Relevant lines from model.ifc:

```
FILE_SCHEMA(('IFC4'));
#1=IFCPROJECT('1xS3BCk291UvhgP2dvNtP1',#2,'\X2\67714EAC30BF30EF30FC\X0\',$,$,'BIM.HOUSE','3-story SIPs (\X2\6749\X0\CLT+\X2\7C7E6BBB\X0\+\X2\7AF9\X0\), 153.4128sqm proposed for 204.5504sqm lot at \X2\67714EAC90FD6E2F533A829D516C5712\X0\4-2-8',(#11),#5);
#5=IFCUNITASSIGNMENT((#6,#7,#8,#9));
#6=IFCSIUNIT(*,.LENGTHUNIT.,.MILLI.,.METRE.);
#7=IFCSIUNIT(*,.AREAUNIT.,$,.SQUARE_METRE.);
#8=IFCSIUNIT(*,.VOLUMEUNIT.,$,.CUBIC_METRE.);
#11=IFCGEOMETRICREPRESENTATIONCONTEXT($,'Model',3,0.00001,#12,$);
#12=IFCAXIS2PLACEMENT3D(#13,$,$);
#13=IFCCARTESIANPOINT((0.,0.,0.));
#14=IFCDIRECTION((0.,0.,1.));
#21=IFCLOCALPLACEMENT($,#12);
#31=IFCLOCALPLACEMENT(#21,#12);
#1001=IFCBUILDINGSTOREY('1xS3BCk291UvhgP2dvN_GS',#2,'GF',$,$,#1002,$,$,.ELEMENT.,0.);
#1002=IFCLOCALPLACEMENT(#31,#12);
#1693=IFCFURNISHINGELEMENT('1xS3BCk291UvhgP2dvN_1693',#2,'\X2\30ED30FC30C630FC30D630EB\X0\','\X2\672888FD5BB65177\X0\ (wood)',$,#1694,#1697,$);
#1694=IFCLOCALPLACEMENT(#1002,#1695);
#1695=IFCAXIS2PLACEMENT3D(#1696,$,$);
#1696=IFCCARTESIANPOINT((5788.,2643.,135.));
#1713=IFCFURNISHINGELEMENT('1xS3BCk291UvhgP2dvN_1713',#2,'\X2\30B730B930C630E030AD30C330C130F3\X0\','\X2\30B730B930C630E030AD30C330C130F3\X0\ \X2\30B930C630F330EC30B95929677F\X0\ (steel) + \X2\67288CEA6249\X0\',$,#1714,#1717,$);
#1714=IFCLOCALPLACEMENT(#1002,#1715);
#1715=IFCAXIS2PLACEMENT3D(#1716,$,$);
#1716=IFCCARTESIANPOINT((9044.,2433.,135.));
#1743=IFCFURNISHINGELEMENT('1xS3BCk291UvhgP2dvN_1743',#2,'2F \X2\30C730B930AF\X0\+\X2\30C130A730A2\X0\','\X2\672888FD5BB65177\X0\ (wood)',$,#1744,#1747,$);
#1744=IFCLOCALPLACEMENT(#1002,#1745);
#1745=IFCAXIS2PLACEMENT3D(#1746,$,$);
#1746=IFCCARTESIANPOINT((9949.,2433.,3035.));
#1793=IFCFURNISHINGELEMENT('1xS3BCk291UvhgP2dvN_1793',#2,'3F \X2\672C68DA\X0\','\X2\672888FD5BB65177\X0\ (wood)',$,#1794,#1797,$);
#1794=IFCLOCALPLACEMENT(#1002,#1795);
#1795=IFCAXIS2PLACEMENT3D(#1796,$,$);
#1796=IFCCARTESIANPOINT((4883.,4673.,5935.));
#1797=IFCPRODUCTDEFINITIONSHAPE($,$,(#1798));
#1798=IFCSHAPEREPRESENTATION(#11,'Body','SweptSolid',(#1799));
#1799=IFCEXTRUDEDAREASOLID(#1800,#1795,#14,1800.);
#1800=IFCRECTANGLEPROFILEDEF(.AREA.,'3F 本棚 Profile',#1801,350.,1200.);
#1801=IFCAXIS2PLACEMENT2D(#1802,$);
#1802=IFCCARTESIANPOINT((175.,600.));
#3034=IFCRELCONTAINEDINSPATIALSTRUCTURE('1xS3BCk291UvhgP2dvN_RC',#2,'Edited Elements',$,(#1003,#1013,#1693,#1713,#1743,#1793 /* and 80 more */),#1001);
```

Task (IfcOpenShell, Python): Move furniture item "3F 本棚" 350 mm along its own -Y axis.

```python
import ifcopenshell
import ifcopenshell.api.geometry
import ifcopenshell.util.placement

model = ifcopenshell.open("model.ifc")

item = model.by_id(1793)
matrix = ifcopenshell.util.placement.get_local_placement(item.ObjectPlacement)
matrix[:3, 3] -= matrix[:3, 1] * 350.0
ifcopenshell.api.geometry.edit_object_placement(model, product=item, matrix=matrix, is_si=False)

print(ifcopenshell.util.placement.get_local_placement(item.ObjectPlacement).round(3) + 0.0)

model.write("model_v2.ifc")
```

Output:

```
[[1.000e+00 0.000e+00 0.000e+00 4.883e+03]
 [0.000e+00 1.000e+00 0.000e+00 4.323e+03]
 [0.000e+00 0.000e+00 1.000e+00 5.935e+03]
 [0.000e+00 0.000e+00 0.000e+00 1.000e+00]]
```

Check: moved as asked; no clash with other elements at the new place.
